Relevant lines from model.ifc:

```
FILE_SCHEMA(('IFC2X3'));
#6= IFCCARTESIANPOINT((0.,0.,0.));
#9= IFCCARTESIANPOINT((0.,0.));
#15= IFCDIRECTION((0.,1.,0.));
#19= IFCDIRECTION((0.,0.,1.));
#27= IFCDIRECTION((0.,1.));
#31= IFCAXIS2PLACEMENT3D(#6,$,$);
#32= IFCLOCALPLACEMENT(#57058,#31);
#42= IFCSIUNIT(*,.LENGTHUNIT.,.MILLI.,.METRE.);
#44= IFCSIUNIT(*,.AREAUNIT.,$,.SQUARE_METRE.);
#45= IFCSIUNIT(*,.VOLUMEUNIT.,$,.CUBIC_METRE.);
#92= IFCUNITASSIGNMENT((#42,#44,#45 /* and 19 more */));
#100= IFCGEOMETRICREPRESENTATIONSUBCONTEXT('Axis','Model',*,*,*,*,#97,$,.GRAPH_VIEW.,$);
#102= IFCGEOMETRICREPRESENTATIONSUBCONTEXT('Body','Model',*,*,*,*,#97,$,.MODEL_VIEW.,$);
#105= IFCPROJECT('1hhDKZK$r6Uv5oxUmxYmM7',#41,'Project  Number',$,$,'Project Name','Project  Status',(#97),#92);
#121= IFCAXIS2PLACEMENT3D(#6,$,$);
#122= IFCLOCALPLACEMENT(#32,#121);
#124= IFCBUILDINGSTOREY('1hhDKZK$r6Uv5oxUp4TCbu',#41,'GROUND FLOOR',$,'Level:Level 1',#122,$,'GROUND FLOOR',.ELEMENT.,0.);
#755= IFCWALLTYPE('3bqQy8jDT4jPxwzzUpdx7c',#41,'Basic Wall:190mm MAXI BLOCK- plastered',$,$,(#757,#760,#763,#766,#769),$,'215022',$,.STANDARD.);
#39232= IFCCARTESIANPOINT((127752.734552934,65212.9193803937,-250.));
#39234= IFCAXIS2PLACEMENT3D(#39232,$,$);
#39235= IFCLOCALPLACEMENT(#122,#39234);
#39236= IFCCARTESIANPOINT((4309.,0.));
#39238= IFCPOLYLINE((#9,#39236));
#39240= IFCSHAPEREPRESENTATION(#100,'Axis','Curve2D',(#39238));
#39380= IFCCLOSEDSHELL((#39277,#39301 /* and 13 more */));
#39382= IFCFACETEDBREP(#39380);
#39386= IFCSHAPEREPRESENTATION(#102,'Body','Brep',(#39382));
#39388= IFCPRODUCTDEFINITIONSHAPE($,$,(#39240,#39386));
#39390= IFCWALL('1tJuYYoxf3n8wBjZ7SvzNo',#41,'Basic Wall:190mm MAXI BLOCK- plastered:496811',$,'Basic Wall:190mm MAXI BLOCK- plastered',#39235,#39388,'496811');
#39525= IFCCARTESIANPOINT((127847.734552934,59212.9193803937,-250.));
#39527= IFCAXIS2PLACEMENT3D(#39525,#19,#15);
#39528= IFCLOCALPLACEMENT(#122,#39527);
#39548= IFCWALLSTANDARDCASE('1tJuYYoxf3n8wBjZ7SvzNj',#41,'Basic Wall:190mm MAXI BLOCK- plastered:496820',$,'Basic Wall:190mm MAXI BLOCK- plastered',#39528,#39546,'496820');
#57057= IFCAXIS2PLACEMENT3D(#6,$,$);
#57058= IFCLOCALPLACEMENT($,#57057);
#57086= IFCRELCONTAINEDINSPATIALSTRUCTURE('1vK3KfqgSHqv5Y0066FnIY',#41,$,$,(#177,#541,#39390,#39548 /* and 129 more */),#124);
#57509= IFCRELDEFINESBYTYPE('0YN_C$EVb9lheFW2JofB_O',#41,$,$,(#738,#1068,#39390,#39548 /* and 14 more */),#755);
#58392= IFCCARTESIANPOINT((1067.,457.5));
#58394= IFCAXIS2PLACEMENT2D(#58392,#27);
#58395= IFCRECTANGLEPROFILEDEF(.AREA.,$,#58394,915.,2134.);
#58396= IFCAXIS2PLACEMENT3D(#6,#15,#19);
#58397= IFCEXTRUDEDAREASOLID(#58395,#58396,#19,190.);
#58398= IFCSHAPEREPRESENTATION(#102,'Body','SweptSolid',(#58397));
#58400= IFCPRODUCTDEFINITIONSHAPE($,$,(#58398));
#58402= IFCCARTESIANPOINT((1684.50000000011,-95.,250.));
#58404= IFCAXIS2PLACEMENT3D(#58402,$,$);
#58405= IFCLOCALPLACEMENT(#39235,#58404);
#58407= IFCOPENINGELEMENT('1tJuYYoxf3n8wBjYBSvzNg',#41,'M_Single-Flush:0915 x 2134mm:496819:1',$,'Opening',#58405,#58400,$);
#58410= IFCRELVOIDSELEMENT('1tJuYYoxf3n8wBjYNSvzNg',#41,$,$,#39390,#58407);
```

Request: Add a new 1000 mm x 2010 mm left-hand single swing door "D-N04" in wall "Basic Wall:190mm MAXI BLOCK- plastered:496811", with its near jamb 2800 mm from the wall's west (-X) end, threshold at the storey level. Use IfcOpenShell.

```python
import numpy as np
import ifcopenshell
import ifcopenshell.api.feature
import ifcopenshell.api.geometry
import ifcopenshell.api.root
import ifcopenshell.api.spatial
import ifcopenshell.api.type
import ifcopenshell.geom
import ifcopenshell.util.element
import ifcopenshell.util.placement
import ifcopenshell.util.representation
import ifcopenshell.util.shape
import ifcopenshell.util.unit

model = ifcopenshell.open("model.ifc")
unit_scale = ifcopenshell.util.unit.calculate_unit_scale(model)
settings = ifcopenshell.geom.settings()


def volume(element):
    """Net volume in cubic metres, openings subtracted."""
    shape = ifcopenshell.geom.create_shape(settings, element)
    return ifcopenshell.util.shape.get_volume(shape.geometry)


wall = model.by_id(39390)
storey = ifcopenshell.util.element.get_container(wall, ifc_class="IfcBuildingStorey")
context = ifcopenshell.util.representation.get_context(model, "Model", "Body", "MODEL_VIEW")
before = volume(wall)

width, height, from_end, sill = 1, 2.01, 2.8, 0.0  # metres

# The wall runs along its own X axis, and the end named is its -X end.
wall_shape = ifcopenshell.geom.create_shape(settings, wall)
x, y, z = ifcopenshell.util.shape.get_vertices(wall_shape.geometry).T
start = x.min() + from_end
face, thickness = float(y.min()), float(y.max() - y.min())
wall_matrix = ifcopenshell.util.placement.get_local_placement(wall.ObjectPlacement)
level = ifcopenshell.util.placement.get_local_placement(storey.ObjectPlacement)[2, 3]


def in_wall(x, y):
    """Placement at x, y metres in the wall's axes, at sill height."""
    matrix = wall_matrix.copy()
    matrix[:, 3] = wall_matrix @ np.array([x / unit_scale, y / unit_scale, 0.0, 1.0])
    matrix[2, 3] = level + sill / unit_scale
    return matrix


# Opening: a box that overshoots both wall faces by 50 mm.
opening = ifcopenshell.api.root.create_entity(model, ifc_class="IfcOpeningElement")
box = ifcopenshell.api.geometry.add_wall_representation(
    model, context=context, length=width, height=height, thickness=thickness + 0.1
)
ifcopenshell.api.geometry.assign_representation(model, product=opening, representation=box)
ifcopenshell.api.geometry.edit_object_placement(model, product=opening, matrix=in_wall(start, face - 0.05), is_si=False)
ifcopenshell.api.feature.add_feature(model, feature=opening, element=wall)

door = ifcopenshell.api.root.create_entity(model, ifc_class="IfcDoor", name="D-N04")
door.OverallWidth, door.OverallHeight = width / unit_scale, height / unit_scale
body = ifcopenshell.api.geometry.add_door_representation(
    model,
    context=context,
    overall_width=door.OverallWidth,
    overall_height=door.OverallHeight,
    operation_type="SINGLE_SWING_LEFT",
    lining_properties={"LiningDepth": thickness / unit_scale, "ThresholdDepth": thickness / unit_scale},
)
ifcopenshell.api.geometry.assign_representation(model, product=door, representation=body)
ifcopenshell.api.spatial.assign_container(model, products=[door], relating_structure=storey)
fills = ifcopenshell.api.feature.add_filling(model, opening=opening, element=door)
fills.OwnerHistory = door.OwnerHistory  # required in IFC2X3

# IFC2X3 keeps the operation on the door style.
style = ifcopenshell.api.root.create_entity(model, ifc_class="IfcDoorStyle", name="D-N04")
style.OperationType, style.ConstructionType = "SINGLE_SWING_LEFT", "NOTDEFINED"
style.ParameterTakesPrecedence = style.Sizeable = False
ifcopenshell.api.type.assign_type(model, related_objects=[door], relating_type=style)

# The lining spans the wall, so the door starts at the wall face.
ifcopenshell.api.geometry.edit_object_placement(model, product=door, matrix=in_wall(start, face), is_si=False)

after = volume(wall)

print(f"wall volume {before:.3f} -> {after:.3f} m3")

model.write("model_v2.ifc")
```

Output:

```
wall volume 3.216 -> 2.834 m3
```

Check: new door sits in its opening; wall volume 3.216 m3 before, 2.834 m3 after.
